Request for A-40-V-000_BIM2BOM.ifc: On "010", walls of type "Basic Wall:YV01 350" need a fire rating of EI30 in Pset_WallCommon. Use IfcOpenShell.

First a look at what the model holds.

```python
import ifcopenshell
import ifcopenshell.util.element

model = ifcopenshell.open("A-40-V-000_BIM2BOM.ifc")
print(model.schema)
storey = next(s for s in model.by_type("IfcBuildingStorey") if s.Name == "010")
walls = [e for e in ifcopenshell.util.element.get_decomposition(storey) if e.is_a("IfcWall")]
seen = {}
for e in walls:
    element_type = ifcopenshell.util.element.get_type(e)
    key = (element_type.Name if element_type != e and element_type else None, ifcopenshell.util.element.get_pset(e, "Pset_WallCommon", "FireRating"))
    seen[key] = seen.get(key, 0) + 1
for (name, value), count in sorted(seen.items(), key=str):
    print(count, "x", name, "|", value)
```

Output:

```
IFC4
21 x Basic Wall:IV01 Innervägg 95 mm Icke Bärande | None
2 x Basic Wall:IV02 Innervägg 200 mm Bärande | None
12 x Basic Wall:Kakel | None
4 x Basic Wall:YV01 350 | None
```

```python
import ifcopenshell
import ifcopenshell.api.pset
import ifcopenshell.util.element

model = ifcopenshell.open("A-40-V-000_BIM2BOM.ifc")

storey = next(s for s in model.by_type("IfcBuildingStorey") if s.Name == "010")
walls = [e for e in ifcopenshell.util.element.get_decomposition(storey) if e.is_a("IfcWall")]

count = 0
for e in walls:
    element_type = ifcopenshell.util.element.get_type(e)
    if element_type in (None, e) or element_type.Name != "Basic Wall:YV01 350":
        continue
    # add_pset returns the element's existing set when there is one.
    pset = ifcopenshell.api.pset.add_pset(model, product=e, name="Pset_WallCommon")
    ifcopenshell.api.pset.edit_pset(model, pset=pset, properties={"FireRating": "EI30"})
    count += 1

print(count, "walls updated")

model.write("A-40-V-000_BIM2BOM_edited.ifc")
```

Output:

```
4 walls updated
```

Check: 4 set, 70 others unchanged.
